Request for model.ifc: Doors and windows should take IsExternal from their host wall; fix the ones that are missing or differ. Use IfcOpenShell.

First a look at what the model holds.

```python
import ifcopenshell
import ifcopenshell.util.element

model = ifcopenshell.open("model.ifc")
print(model.schema)
seen = {}
for e in model.by_type("IfcDoor") + model.by_type("IfcWindow"):
    if not e.FillsVoids:
        continue
    host = e.FillsVoids[0].RelatingOpeningElement.VoidsElements[0].RelatingBuildingElement
    own = ifcopenshell.util.element.get_pset(e, f"Pset_{e.is_a()[3:].removesuffix('StandardCase')}Common", "IsExternal")
    wall = ifcopenshell.util.element.get_pset(host, "Pset_WallCommon", "IsExternal")
    seen[e.is_a(), own, wall] = seen.get((e.is_a(), own, wall), 0) + 1
for (cls, own, wall), count in sorted(seen.items(), key=str):
    print(count, cls, "IsExternal:", own, "| host wall:", wall)
```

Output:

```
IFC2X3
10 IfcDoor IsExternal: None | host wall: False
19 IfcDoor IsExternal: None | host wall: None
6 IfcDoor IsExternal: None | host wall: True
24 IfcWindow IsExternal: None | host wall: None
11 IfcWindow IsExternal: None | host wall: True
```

```python
import ifcopenshell
import ifcopenshell.api.pset
import ifcopenshell.util.element

model = ifcopenshell.open("model.ifc")

count = 0
for ifc_class, pset_name in (("IfcDoor", "Pset_DoorCommon"), ("IfcWindow", "Pset_WindowCommon")):
    for e in model.by_type(ifc_class):
        if not e.FillsVoids:
            continue
        host = e.FillsVoids[0].RelatingOpeningElement.VoidsElements[0].RelatingBuildingElement
        external = ifcopenshell.util.element.get_pset(host, "Pset_WallCommon", "IsExternal")
        if external is None or ifcopenshell.util.element.get_pset(e, pset_name, "IsExternal") == external:
            continue
        pset = ifcopenshell.api.pset.add_pset(model, product=e, name=pset_name)
        ifcopenshell.api.pset.edit_pset(model, pset=pset, properties={"IsExternal": external})
        count += 1

print(count, "updated")

model.write("model_edited.ifc")
```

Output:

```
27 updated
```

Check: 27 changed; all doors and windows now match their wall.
